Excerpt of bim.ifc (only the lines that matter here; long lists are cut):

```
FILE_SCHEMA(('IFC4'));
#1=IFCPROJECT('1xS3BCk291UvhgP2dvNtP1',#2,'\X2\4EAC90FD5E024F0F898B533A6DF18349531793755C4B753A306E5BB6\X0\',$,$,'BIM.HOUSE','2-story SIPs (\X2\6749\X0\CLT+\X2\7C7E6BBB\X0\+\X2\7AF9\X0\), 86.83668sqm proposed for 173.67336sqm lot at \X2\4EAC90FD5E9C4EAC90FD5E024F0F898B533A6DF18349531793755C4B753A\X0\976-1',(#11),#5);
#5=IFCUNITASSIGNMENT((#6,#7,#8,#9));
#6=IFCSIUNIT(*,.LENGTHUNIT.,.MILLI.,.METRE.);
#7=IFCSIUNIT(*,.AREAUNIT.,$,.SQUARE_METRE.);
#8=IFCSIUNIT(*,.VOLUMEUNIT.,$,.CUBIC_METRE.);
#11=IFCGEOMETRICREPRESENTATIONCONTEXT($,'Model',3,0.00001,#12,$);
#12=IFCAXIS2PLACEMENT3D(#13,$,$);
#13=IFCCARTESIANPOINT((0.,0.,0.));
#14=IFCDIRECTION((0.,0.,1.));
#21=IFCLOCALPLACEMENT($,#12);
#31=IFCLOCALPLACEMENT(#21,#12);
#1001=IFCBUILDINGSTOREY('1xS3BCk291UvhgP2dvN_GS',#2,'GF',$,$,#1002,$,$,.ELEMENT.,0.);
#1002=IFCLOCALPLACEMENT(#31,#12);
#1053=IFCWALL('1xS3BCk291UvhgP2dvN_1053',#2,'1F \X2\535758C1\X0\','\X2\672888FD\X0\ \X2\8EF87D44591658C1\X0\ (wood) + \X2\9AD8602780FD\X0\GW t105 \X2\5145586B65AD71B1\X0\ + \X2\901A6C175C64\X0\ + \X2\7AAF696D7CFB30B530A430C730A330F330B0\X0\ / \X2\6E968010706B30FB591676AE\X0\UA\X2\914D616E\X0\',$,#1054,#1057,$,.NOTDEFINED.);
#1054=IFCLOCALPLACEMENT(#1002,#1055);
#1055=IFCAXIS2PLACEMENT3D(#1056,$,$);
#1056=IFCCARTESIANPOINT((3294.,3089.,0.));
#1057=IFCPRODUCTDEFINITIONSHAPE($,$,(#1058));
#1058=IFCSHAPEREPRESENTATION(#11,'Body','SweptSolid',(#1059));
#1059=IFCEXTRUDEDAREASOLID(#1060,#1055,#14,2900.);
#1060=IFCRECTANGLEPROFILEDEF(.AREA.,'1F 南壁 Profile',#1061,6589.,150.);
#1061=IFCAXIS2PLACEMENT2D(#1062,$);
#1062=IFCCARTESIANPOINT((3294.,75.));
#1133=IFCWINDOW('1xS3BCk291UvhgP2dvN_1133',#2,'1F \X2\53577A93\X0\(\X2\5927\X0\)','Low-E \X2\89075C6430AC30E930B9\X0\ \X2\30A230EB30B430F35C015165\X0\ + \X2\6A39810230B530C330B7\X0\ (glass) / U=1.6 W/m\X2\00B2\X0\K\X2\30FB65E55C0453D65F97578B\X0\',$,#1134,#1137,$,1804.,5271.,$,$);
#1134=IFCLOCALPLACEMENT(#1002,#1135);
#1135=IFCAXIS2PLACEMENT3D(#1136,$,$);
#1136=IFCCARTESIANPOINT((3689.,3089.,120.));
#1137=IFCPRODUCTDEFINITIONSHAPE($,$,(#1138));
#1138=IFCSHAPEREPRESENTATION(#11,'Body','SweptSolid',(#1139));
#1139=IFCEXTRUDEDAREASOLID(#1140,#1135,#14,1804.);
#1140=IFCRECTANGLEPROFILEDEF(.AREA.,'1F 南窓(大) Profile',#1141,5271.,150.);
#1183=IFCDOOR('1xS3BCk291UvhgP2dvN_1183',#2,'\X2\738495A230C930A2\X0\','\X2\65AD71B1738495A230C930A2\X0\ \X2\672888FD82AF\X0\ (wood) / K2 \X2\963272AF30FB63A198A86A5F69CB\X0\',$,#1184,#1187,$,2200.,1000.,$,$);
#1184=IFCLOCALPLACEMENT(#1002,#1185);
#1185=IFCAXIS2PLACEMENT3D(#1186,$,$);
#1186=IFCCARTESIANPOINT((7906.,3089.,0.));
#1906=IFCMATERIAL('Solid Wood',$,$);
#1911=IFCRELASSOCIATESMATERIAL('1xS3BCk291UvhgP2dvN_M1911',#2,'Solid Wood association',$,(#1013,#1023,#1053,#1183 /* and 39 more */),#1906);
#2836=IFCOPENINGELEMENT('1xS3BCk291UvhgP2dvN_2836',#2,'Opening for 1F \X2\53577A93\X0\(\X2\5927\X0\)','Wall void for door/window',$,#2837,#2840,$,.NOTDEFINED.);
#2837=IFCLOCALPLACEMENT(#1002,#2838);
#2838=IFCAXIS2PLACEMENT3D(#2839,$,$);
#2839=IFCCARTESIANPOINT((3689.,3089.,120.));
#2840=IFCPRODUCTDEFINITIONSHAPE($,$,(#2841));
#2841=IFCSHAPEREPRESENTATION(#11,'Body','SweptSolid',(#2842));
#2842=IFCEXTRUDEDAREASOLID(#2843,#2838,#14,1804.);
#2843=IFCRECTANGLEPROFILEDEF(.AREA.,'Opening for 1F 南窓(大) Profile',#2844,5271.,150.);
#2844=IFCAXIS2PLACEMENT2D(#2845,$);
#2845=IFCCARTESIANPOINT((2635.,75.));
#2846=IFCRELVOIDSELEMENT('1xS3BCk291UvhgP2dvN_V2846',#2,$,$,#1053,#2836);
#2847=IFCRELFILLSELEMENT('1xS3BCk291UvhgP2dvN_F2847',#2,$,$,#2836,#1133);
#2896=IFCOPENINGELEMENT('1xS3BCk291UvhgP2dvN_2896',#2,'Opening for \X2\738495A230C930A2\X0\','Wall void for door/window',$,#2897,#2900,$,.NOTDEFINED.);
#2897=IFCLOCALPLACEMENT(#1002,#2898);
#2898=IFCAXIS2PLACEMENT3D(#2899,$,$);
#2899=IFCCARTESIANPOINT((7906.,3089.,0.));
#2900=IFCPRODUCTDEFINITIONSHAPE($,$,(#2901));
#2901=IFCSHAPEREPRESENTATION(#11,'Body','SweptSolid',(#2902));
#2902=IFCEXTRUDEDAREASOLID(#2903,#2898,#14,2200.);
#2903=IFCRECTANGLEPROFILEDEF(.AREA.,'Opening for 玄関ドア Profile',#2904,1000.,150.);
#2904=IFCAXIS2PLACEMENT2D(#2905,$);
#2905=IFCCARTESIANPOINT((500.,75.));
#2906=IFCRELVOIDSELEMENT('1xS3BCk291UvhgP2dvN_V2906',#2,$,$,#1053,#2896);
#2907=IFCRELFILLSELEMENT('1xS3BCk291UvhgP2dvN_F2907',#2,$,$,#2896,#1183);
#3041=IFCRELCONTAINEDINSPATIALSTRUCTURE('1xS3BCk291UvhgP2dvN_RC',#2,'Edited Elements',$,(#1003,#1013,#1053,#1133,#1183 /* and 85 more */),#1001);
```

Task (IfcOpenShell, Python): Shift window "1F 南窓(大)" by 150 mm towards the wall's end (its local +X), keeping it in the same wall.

```python
import ifcopenshell
import ifcopenshell.api.geometry
import ifcopenshell.util.placement
import ifcopenshell.util.unit

model = ifcopenshell.open("bim.ifc")
unit_scale = ifcopenshell.util.unit.calculate_unit_scale(model)

window = model.by_guid("1xS3BCk291UvhgP2dvN_1133")
opening = window.FillsVoids[0].RelatingOpeningElement
wall = opening.VoidsElements[0].RelatingBuildingElement

wall_matrix = ifcopenshell.util.placement.get_local_placement(wall.ObjectPlacement)
shift = wall_matrix[:3, 0] * 0.15 / unit_scale
before = ifcopenshell.util.placement.get_local_placement(window.ObjectPlacement)[:3, 3].copy()

# The window is not placed relative to its opening, so move both.
for product in (opening, window):
    matrix = ifcopenshell.util.placement.get_local_placement(product.ObjectPlacement)
    matrix[:3, 3] += shift
    ifcopenshell.api.geometry.edit_object_placement(model, product=product, matrix=matrix, is_si=False)

after = ifcopenshell.util.placement.get_local_placement(window.ObjectPlacement)[:3, 3]
print("window moved by", (after - before).round(3) + 0.0)

model.write("bim_edited.ifc")
```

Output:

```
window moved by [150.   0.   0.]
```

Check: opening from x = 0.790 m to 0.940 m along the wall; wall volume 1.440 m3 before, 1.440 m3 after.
